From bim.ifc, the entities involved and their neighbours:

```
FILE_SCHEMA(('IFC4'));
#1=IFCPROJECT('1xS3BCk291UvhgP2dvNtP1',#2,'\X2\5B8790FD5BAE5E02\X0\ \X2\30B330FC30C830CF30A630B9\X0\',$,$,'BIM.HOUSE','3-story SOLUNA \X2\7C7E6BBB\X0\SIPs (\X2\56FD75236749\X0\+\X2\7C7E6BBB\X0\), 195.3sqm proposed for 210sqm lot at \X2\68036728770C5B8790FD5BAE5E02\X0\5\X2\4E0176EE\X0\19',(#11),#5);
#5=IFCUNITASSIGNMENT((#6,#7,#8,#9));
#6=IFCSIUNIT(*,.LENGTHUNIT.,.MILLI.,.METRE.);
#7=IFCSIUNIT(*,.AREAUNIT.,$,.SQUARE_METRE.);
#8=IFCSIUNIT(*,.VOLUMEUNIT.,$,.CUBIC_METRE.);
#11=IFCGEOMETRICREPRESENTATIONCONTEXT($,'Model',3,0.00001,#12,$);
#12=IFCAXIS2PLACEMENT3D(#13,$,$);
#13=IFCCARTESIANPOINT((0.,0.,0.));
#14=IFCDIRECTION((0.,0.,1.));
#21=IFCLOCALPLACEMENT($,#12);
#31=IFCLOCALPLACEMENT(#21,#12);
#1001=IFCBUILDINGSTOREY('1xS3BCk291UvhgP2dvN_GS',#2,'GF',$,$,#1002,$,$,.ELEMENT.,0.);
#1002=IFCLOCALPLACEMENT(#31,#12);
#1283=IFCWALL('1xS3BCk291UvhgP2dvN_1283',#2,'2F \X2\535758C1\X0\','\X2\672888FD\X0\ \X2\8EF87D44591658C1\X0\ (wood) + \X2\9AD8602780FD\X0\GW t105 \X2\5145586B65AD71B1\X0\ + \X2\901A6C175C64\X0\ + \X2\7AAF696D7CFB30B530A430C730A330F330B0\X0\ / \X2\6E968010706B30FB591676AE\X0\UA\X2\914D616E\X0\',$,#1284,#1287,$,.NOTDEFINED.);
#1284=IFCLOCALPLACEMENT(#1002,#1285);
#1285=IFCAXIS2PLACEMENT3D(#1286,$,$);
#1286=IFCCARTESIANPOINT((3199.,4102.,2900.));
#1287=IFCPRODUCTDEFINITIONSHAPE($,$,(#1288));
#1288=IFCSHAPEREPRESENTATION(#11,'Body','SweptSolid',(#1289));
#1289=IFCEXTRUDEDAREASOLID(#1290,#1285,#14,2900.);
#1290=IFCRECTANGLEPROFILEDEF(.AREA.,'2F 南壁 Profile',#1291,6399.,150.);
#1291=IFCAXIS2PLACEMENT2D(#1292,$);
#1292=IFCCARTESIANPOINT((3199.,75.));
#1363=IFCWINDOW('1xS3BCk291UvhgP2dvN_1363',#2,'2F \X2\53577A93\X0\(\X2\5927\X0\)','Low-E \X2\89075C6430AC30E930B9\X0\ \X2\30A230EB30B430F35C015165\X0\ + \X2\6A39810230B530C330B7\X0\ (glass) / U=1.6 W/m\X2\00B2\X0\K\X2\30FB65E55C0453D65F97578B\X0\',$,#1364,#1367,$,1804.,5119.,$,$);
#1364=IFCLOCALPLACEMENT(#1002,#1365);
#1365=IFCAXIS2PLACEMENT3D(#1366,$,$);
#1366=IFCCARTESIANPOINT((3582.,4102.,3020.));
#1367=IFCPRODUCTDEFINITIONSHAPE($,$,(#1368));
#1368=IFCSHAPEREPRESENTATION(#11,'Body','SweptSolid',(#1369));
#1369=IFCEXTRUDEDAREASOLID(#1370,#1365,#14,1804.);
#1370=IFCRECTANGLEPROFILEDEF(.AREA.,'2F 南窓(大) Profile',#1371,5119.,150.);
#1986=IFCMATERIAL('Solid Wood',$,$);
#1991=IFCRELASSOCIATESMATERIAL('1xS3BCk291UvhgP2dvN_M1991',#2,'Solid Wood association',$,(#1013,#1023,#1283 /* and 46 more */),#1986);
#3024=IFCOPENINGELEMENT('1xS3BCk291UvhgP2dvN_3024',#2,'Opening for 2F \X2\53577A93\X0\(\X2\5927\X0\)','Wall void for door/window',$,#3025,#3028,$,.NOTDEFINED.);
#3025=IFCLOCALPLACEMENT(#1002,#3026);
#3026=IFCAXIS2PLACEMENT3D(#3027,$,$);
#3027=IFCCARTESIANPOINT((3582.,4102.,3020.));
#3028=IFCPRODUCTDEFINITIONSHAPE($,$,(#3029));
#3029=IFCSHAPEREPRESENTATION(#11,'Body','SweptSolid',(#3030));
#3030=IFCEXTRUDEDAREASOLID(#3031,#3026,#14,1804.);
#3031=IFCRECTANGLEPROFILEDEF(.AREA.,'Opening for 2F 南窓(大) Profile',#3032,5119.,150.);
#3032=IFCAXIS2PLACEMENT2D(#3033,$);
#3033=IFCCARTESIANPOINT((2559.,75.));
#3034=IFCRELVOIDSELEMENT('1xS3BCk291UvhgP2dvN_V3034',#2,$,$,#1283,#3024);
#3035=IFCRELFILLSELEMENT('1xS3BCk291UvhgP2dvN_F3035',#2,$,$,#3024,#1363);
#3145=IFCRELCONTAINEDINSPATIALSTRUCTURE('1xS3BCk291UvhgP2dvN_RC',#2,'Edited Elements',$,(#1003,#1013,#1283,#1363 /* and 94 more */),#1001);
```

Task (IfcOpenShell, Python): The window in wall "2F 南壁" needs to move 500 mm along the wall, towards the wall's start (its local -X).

```python
import ifcopenshell
import ifcopenshell.api.geometry
import ifcopenshell.util.placement

model = ifcopenshell.open("bim.ifc")

window = model.by_guid("1xS3BCk291UvhgP2dvN_1363")
opening = window.FillsVoids[0].RelatingOpeningElement
wall = opening.VoidsElements[0].RelatingBuildingElement

wall_matrix = ifcopenshell.util.placement.get_local_placement(wall.ObjectPlacement)
shift = wall_matrix[:3, 0] * -500.0
before = ifcopenshell.util.placement.get_local_placement(window.ObjectPlacement)[:3, 3].copy()

# The window is not placed relative to its opening, so move both.
for product in (opening, window):
    matrix = ifcopenshell.util.placement.get_local_placement(product.ObjectPlacement)
    matrix[:3, 3] += shift
    ifcopenshell.api.geometry.edit_object_placement(model, product=product, matrix=matrix, is_si=False)

after = ifcopenshell.util.placement.get_local_placement(window.ObjectPlacement)[:3, 3]
print("window moved by", (after - before).round(3) + 0.0)

model.write("bim-out.ifc")
```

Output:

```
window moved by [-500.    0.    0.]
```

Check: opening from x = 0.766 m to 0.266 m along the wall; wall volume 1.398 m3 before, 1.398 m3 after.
